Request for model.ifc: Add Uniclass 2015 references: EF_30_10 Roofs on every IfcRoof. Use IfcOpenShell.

First a look at what the model holds.

```python
import ifcopenshell

model = ifcopenshell.open("model.ifc")
print(model.schema)
print("classifications:", [c.Name for c in model.by_type("IfcClassification")])
for ifc_class in ("IfcDoor", "IfcRoof", "IfcStair", "IfcWall", "IfcWindow"):
    print(ifc_class, len(model.by_type(ifc_class)))
```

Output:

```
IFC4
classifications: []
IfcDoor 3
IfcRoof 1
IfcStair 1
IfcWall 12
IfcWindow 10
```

```python
import ifcopenshell
import ifcopenshell.api.classification

model = ifcopenshell.open("model.ifc")

system = ifcopenshell.api.classification.add_classification(model, classification="Uniclass 2015")

codes = {
    "IfcRoof": ("EF_30_10", "Roofs"),
}
for ifc_class, (code, name) in codes.items():
    products = model.by_type(ifc_class)
    ifcopenshell.api.classification.add_reference(
        model, products=products, classification=system, identification=code, name=name
    )
    print(code, len(products))

model.write("model_edited.ifc")
```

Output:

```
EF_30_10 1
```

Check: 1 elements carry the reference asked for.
